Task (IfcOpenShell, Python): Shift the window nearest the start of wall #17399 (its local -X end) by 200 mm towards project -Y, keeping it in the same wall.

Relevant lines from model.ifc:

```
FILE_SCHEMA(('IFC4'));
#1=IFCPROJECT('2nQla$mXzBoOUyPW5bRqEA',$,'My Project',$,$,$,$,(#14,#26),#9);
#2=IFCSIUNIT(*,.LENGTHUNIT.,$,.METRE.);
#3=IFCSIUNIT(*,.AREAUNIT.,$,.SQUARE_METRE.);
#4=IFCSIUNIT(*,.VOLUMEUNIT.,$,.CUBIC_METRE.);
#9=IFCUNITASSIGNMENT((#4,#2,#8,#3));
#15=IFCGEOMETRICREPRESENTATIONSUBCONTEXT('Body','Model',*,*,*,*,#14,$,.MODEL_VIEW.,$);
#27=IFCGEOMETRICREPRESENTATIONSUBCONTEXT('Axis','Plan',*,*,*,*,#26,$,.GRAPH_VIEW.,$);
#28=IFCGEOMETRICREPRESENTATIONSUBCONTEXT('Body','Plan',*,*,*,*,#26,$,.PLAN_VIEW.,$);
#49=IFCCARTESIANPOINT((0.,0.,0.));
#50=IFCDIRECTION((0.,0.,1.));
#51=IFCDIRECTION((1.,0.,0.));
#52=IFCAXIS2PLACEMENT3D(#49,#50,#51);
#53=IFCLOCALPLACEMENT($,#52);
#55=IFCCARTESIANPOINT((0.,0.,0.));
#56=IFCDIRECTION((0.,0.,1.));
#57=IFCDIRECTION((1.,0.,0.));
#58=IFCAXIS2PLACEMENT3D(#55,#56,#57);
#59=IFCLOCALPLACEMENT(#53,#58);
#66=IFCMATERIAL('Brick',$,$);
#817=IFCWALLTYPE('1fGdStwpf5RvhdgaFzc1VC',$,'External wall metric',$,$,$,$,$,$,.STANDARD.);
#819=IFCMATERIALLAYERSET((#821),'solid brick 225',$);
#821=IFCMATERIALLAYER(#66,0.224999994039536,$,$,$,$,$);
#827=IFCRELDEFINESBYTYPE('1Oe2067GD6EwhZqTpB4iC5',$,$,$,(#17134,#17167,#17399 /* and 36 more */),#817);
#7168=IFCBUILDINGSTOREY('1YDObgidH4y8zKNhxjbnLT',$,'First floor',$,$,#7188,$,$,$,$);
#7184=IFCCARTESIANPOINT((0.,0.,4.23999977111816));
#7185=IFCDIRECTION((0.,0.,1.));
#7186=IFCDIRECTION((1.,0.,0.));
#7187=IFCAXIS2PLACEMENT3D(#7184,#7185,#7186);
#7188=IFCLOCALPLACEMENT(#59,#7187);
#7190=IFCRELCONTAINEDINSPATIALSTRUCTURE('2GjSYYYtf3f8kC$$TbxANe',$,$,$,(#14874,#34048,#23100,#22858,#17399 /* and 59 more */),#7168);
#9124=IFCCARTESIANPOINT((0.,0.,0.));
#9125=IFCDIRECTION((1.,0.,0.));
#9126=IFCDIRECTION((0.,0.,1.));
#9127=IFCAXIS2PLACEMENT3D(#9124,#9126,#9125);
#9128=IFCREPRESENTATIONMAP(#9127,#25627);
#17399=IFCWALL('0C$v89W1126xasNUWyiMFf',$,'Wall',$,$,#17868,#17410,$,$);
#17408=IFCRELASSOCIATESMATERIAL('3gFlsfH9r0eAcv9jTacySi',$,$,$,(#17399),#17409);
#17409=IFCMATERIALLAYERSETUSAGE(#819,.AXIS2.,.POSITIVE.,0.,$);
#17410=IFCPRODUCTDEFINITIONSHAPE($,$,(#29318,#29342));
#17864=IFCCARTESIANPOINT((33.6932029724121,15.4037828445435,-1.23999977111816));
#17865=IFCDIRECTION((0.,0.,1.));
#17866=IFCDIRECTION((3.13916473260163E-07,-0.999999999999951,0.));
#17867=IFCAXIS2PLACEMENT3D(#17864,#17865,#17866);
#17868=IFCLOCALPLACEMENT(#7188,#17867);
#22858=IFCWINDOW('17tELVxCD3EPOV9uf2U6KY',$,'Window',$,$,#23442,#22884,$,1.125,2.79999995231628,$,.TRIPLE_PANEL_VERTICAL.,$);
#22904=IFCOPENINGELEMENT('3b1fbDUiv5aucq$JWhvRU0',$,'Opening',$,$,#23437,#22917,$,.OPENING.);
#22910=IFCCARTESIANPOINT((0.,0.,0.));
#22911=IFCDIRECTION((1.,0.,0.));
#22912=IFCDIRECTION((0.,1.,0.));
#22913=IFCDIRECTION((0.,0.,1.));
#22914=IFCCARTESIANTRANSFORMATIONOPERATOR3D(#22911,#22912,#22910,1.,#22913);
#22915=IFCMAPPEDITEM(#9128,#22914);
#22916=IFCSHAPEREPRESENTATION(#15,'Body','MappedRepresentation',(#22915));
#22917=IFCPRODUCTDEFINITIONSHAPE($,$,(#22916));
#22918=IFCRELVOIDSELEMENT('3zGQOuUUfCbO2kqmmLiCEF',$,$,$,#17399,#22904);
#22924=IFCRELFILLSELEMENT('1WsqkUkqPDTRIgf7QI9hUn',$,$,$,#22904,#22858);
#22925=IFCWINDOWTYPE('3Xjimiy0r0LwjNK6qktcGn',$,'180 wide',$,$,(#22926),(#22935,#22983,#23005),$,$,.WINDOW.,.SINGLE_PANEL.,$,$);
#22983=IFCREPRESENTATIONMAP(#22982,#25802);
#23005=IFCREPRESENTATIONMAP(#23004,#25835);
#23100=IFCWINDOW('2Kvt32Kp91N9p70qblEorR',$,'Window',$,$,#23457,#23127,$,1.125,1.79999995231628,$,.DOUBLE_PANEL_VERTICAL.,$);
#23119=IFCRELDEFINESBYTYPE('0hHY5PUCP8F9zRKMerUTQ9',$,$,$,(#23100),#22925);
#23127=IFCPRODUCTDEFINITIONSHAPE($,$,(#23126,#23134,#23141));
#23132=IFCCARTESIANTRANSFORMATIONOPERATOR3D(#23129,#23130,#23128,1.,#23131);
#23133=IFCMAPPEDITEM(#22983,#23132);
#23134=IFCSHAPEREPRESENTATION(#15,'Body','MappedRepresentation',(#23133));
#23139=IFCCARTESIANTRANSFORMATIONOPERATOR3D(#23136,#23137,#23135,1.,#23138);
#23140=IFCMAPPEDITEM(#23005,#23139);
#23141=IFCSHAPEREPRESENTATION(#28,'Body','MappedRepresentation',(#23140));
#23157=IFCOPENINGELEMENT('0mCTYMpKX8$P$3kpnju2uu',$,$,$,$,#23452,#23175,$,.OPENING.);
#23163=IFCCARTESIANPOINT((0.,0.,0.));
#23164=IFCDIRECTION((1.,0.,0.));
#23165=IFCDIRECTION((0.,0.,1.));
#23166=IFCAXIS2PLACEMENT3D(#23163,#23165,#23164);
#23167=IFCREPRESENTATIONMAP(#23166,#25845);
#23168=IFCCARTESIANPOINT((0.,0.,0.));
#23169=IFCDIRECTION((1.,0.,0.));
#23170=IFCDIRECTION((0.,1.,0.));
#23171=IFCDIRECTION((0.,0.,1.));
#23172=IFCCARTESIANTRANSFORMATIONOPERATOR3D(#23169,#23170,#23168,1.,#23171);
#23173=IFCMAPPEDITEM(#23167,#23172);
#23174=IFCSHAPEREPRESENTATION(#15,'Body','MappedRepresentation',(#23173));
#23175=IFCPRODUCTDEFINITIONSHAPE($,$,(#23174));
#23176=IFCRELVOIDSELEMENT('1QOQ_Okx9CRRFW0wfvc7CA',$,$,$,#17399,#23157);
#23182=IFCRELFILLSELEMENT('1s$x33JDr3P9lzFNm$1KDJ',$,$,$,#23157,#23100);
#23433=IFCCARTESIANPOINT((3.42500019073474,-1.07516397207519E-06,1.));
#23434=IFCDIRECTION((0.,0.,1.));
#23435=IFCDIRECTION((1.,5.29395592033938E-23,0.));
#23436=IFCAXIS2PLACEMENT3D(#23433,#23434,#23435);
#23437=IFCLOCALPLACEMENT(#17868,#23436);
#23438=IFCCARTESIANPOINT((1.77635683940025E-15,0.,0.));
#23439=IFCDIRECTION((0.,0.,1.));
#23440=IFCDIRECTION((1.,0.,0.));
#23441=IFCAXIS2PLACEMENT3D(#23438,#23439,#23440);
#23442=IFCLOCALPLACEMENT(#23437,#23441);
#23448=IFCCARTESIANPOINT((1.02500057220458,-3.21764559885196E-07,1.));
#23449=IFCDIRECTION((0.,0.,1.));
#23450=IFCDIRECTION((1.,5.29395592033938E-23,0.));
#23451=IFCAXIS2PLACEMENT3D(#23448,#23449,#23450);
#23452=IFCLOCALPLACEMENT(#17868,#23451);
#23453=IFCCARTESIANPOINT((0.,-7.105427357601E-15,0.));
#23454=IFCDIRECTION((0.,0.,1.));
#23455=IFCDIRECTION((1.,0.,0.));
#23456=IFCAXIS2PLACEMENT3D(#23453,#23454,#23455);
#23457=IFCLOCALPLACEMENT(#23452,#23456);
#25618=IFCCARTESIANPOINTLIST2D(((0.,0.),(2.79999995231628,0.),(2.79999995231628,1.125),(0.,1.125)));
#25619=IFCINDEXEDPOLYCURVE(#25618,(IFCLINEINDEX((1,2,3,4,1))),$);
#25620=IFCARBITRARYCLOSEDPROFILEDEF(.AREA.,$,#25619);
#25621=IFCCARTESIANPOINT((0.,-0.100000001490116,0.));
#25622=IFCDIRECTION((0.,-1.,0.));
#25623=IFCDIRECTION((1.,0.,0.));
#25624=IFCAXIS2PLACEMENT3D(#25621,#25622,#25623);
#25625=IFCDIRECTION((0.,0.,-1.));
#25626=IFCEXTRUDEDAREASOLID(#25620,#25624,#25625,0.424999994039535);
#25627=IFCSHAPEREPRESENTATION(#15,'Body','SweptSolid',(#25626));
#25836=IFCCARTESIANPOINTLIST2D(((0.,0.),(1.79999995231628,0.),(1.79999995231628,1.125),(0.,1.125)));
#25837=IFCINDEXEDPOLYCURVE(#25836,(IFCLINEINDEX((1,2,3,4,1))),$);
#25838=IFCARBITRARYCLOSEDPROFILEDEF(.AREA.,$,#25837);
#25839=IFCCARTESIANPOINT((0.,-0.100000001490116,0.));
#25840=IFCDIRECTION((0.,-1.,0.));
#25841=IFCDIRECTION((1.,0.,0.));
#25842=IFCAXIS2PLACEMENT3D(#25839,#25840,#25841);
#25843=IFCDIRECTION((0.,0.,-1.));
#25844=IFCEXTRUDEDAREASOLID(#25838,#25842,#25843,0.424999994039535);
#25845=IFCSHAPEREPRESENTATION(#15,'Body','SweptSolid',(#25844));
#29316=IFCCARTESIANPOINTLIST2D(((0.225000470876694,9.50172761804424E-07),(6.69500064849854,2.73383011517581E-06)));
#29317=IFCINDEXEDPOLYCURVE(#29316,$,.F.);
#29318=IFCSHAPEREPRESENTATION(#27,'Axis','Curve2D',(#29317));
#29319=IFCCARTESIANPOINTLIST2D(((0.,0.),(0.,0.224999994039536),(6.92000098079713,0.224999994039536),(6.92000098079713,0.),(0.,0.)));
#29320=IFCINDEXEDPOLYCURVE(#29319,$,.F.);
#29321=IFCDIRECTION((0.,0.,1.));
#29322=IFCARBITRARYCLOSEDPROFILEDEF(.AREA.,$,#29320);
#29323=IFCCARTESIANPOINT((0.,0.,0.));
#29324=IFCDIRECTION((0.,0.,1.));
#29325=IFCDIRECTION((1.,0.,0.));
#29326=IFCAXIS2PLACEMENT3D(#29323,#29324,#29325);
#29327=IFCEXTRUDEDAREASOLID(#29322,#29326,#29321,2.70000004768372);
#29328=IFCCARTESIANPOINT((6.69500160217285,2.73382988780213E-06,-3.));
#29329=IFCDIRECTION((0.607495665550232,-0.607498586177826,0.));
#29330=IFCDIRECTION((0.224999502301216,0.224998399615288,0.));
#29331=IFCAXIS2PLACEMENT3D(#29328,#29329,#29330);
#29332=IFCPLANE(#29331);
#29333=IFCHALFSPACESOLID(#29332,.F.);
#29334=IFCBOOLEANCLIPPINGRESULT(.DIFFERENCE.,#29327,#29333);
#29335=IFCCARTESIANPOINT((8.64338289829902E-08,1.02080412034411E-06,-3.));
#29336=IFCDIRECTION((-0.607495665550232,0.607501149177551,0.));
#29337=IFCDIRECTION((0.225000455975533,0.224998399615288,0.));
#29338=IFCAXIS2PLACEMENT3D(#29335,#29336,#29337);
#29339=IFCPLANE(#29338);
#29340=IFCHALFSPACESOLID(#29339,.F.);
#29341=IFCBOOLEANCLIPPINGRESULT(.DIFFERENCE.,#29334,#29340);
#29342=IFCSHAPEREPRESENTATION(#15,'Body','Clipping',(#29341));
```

```python
import ifcopenshell
import ifcopenshell.api.geometry
import ifcopenshell.util.placement
import ifcopenshell.util.unit

model = ifcopenshell.open("model.ifc")
unit_scale = ifcopenshell.util.unit.calculate_unit_scale(model)

window = model.by_guid("2Kvt32Kp91N9p70qblEorR")
opening = window.FillsVoids[0].RelatingOpeningElement
wall = opening.VoidsElements[0].RelatingBuildingElement

wall_matrix = ifcopenshell.util.placement.get_local_placement(wall.ObjectPlacement)
shift = wall_matrix[:3, 0] * 0.2 / unit_scale
before = ifcopenshell.util.placement.get_local_placement(window.ObjectPlacement)[:3, 3].copy()

# The window is placed relative to its opening, so it follows when the opening moves.
matrix = ifcopenshell.util.placement.get_local_placement(opening.ObjectPlacement)
matrix[:3, 3] += shift
ifcopenshell.api.geometry.edit_object_placement(
    model, product=opening, matrix=matrix, is_si=False, should_transform_children=True
)

after = ifcopenshell.util.placement.get_local_placement(window.ObjectPlacement)[:3, 3]
print("window moved by", (after - before).round(3) + 0.0)

model.write("model_rev.ifc")
```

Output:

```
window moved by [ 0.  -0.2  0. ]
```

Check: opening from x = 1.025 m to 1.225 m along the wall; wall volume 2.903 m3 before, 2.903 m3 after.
